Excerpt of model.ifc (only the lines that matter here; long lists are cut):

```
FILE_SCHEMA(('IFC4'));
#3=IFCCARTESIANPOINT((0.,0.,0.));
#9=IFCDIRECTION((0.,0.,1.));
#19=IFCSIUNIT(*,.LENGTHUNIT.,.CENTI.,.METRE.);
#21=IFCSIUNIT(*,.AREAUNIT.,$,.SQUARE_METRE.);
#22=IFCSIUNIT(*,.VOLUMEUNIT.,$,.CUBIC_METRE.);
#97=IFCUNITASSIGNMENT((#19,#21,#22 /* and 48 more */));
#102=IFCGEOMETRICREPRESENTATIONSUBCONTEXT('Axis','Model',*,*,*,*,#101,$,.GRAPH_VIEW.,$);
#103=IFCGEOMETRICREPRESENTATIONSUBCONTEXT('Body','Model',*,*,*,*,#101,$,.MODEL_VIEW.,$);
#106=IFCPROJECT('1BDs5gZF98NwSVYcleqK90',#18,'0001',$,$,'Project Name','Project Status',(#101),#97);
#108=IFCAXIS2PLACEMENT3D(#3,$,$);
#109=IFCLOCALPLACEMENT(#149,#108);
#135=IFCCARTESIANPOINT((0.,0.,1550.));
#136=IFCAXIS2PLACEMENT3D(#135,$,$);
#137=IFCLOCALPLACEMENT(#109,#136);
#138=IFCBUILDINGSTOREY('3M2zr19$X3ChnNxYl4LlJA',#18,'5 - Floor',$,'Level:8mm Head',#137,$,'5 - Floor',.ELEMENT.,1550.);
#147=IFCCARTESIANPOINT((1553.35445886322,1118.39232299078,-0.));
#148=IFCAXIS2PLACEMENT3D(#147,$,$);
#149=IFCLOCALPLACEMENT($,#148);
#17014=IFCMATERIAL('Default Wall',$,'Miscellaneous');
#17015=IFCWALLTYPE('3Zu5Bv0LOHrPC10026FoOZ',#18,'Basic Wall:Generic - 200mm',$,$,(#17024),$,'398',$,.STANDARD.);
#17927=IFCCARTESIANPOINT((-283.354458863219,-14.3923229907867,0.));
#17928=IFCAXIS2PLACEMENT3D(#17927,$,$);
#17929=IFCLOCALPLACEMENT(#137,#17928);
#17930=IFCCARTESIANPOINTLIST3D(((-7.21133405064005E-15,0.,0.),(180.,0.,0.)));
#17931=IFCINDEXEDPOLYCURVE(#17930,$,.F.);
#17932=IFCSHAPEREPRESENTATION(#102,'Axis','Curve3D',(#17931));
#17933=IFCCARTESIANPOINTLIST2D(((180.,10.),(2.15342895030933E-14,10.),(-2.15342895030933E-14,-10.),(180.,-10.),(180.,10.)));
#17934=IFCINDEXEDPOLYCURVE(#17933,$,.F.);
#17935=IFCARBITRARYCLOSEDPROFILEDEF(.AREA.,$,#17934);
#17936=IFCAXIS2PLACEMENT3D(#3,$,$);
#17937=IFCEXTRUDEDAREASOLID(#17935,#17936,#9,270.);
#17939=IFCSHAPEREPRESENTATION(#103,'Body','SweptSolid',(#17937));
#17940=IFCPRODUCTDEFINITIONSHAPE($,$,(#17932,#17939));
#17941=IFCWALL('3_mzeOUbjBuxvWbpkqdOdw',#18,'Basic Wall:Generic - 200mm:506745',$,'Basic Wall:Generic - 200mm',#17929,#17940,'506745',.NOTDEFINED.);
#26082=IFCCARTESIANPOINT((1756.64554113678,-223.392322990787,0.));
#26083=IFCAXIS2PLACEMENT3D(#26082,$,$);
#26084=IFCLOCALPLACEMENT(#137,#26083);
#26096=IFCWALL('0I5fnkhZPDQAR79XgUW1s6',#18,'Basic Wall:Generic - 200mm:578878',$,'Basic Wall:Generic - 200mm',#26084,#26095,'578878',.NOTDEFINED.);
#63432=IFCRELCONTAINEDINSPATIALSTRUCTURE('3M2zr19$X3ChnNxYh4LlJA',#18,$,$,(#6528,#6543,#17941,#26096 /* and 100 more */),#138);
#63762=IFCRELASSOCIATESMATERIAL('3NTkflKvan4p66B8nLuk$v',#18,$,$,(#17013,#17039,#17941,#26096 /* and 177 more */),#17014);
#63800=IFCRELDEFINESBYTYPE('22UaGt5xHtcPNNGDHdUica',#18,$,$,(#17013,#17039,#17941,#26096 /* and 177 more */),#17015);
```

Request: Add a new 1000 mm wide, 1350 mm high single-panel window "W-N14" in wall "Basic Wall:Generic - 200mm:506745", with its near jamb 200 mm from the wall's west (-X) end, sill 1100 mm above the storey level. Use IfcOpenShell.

```python
import numpy as np
import ifcopenshell
import ifcopenshell.api.feature
import ifcopenshell.api.geometry
import ifcopenshell.api.root
import ifcopenshell.api.spatial
import ifcopenshell.geom
import ifcopenshell.util.element
import ifcopenshell.util.placement
import ifcopenshell.util.representation
import ifcopenshell.util.shape
import ifcopenshell.util.unit

model = ifcopenshell.open("model.ifc")
unit_scale = ifcopenshell.util.unit.calculate_unit_scale(model)
settings = ifcopenshell.geom.settings()


def volume(element):
    """Net volume in cubic metres, openings subtracted."""
    shape = ifcopenshell.geom.create_shape(settings, element)
    return ifcopenshell.util.shape.get_volume(shape.geometry)


wall = model.by_guid("3_mzeOUbjBuxvWbpkqdOdw")
storey = ifcopenshell.util.element.get_container(wall, ifc_class="IfcBuildingStorey")
context = ifcopenshell.util.representation.get_context(model, "Model", "Body", "MODEL_VIEW")
before = volume(wall)

width, height, from_end, sill = 1, 1.35, 0.2, 1.1  # metres

# The wall runs along its own X axis, and the end named is its -X end.
wall_shape = ifcopenshell.geom.create_shape(settings, wall)
x, y, z = ifcopenshell.util.shape.get_vertices(wall_shape.geometry).T
start = x.min() + from_end
face, thickness = float(y.min()), float(y.max() - y.min())
wall_matrix = ifcopenshell.util.placement.get_local_placement(wall.ObjectPlacement)
level = ifcopenshell.util.placement.get_local_placement(storey.ObjectPlacement)[2, 3]


def in_wall(x, y):
    """Placement at x, y metres in the wall's axes, at sill height."""
    matrix = wall_matrix.copy()
    matrix[:, 3] = wall_matrix @ np.array([x / unit_scale, y / unit_scale, 0.0, 1.0])
    matrix[2, 3] = level + sill / unit_scale
    return matrix


# Opening: a box that overshoots both wall faces by 50 mm.
opening = ifcopenshell.api.root.create_entity(model, ifc_class="IfcOpeningElement", predefined_type="OPENING")
box = ifcopenshell.api.geometry.add_wall_representation(
    model, context=context, length=width, height=height, thickness=thickness + 0.1
)
ifcopenshell.api.geometry.assign_representation(model, product=opening, representation=box)
ifcopenshell.api.geometry.edit_object_placement(model, product=opening, matrix=in_wall(start, face - 0.05), is_si=False)
ifcopenshell.api.feature.add_feature(model, feature=opening, element=wall)

window = ifcopenshell.api.root.create_entity(model, ifc_class="IfcWindow", name="W-N14", predefined_type="WINDOW")
window.OverallWidth, window.OverallHeight = width / unit_scale, height / unit_scale
window.PartitioningType = "SINGLE_PANEL"
body = ifcopenshell.api.geometry.add_window_representation(
    model,
    context=context,
    overall_width=window.OverallWidth,
    overall_height=window.OverallHeight,
    partition_type="SINGLE_PANEL",
)
ifcopenshell.api.geometry.assign_representation(model, product=window, representation=body)
ifcopenshell.api.spatial.assign_container(model, products=[window], relating_structure=storey)
ifcopenshell.api.feature.add_filling(model, opening=opening, element=window)

# Centre the window in the wall's thickness.
ifcopenshell.api.geometry.edit_object_placement(model, product=window, matrix=in_wall(start, face), is_si=False)
window_shape = ifcopenshell.geom.create_shape(settings, window)
depth = ifcopenshell.util.shape.get_vertices(window_shape.geometry)[:, 1]
offset = face + thickness / 2 - (depth.min() + depth.max()) / 2
ifcopenshell.api.geometry.edit_object_placement(model, product=window, matrix=in_wall(start, offset), is_si=False)

after = volume(wall)

print(f"wall volume {before:.3f} -> {after:.3f} m3")

model.write("model_updated.ifc")
```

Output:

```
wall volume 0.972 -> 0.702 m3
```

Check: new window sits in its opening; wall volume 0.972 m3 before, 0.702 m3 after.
